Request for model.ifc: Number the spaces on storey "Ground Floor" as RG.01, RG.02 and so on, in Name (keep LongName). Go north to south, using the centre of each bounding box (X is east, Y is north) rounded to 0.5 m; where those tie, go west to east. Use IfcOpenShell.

First a look at what the model holds.

```python
import ifcopenshell
import ifcopenshell.util.element
import ifcopenshell.util.placement

model = ifcopenshell.open("model.ifc")
print(model.schema)
storey = next(s for s in model.by_type("IfcBuildingStorey") if s.Name == "Ground Floor")
spaces = [e for e in ifcopenshell.util.element.get_decomposition(storey) if e.is_a("IfcSpace")]
for e in sorted(spaces, key=lambda e: e.id()):
    origin = ifcopenshell.util.placement.get_local_placement(e.ObjectPlacement)[:3, 3]
    print(e.id(), e.Name, e.LongName, origin.round(2) + 0.0, sep=" | ")
```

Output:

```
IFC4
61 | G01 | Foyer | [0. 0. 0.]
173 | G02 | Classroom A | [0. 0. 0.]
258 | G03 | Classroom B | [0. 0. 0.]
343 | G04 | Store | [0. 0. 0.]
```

```python
import ifcopenshell
import ifcopenshell.geom
import ifcopenshell.util.element
import ifcopenshell.util.shape

model = ifcopenshell.open("model.ifc")
settings = ifcopenshell.geom.settings()
settings.set("use-world-coords", True)


def centre(element):
    shape = ifcopenshell.geom.create_shape(settings, element)
    return ifcopenshell.util.shape.get_bbox_centroid(shape.geometry)


storey = next(s for s in model.by_type("IfcBuildingStorey") if s.Name == "Ground Floor")
spaces = [e for e in ifcopenshell.util.element.get_decomposition(storey) if e.is_a("IfcSpace")]

# Insertion points can sit at a corner or the storey origin, so sort by the geometry (in metres).
centres = {e: centre(e) for e in spaces}
spaces.sort(key=lambda e: (-round(centres[e][1] / 0.5), centres[e][0]))

for i, e in enumerate(spaces, start=1):
    number = f"RG.{i:02d}"
    e.Name = number
    print(e.id(), number)

model.write("model_edited.ifc")
```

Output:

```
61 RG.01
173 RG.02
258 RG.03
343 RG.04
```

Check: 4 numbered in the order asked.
